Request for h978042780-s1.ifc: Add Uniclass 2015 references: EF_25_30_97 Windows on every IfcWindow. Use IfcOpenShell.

First a look at what the model holds.

```python
import ifcopenshell

model = ifcopenshell.open("h978042780-s1.ifc")
print(model.schema)
print("classifications:", [c.Name for c in model.by_type("IfcClassification")])
for ifc_class in ("IfcDoor", "IfcRoof", "IfcStair", "IfcWall", "IfcWindow"):
    print(ifc_class, len(model.by_type(ifc_class)))
```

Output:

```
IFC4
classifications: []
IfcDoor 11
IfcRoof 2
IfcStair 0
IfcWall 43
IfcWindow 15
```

```python
import ifcopenshell
import ifcopenshell.api.classification

model = ifcopenshell.open("h978042780-s1.ifc")

system = ifcopenshell.api.classification.add_classification(model, classification="Uniclass 2015")

codes = {
    "IfcWindow": ("EF_25_30_97", "Windows"),
}
for ifc_class, (code, name) in codes.items():
    products = model.by_type(ifc_class)
    ifcopenshell.api.classification.add_reference(
        model, products=products, classification=system, identification=code, name=name
    )
    print(code, len(products))

model.write("h978042780-s1_edited.ifc")
```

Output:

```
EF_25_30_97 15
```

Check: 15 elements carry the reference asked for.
